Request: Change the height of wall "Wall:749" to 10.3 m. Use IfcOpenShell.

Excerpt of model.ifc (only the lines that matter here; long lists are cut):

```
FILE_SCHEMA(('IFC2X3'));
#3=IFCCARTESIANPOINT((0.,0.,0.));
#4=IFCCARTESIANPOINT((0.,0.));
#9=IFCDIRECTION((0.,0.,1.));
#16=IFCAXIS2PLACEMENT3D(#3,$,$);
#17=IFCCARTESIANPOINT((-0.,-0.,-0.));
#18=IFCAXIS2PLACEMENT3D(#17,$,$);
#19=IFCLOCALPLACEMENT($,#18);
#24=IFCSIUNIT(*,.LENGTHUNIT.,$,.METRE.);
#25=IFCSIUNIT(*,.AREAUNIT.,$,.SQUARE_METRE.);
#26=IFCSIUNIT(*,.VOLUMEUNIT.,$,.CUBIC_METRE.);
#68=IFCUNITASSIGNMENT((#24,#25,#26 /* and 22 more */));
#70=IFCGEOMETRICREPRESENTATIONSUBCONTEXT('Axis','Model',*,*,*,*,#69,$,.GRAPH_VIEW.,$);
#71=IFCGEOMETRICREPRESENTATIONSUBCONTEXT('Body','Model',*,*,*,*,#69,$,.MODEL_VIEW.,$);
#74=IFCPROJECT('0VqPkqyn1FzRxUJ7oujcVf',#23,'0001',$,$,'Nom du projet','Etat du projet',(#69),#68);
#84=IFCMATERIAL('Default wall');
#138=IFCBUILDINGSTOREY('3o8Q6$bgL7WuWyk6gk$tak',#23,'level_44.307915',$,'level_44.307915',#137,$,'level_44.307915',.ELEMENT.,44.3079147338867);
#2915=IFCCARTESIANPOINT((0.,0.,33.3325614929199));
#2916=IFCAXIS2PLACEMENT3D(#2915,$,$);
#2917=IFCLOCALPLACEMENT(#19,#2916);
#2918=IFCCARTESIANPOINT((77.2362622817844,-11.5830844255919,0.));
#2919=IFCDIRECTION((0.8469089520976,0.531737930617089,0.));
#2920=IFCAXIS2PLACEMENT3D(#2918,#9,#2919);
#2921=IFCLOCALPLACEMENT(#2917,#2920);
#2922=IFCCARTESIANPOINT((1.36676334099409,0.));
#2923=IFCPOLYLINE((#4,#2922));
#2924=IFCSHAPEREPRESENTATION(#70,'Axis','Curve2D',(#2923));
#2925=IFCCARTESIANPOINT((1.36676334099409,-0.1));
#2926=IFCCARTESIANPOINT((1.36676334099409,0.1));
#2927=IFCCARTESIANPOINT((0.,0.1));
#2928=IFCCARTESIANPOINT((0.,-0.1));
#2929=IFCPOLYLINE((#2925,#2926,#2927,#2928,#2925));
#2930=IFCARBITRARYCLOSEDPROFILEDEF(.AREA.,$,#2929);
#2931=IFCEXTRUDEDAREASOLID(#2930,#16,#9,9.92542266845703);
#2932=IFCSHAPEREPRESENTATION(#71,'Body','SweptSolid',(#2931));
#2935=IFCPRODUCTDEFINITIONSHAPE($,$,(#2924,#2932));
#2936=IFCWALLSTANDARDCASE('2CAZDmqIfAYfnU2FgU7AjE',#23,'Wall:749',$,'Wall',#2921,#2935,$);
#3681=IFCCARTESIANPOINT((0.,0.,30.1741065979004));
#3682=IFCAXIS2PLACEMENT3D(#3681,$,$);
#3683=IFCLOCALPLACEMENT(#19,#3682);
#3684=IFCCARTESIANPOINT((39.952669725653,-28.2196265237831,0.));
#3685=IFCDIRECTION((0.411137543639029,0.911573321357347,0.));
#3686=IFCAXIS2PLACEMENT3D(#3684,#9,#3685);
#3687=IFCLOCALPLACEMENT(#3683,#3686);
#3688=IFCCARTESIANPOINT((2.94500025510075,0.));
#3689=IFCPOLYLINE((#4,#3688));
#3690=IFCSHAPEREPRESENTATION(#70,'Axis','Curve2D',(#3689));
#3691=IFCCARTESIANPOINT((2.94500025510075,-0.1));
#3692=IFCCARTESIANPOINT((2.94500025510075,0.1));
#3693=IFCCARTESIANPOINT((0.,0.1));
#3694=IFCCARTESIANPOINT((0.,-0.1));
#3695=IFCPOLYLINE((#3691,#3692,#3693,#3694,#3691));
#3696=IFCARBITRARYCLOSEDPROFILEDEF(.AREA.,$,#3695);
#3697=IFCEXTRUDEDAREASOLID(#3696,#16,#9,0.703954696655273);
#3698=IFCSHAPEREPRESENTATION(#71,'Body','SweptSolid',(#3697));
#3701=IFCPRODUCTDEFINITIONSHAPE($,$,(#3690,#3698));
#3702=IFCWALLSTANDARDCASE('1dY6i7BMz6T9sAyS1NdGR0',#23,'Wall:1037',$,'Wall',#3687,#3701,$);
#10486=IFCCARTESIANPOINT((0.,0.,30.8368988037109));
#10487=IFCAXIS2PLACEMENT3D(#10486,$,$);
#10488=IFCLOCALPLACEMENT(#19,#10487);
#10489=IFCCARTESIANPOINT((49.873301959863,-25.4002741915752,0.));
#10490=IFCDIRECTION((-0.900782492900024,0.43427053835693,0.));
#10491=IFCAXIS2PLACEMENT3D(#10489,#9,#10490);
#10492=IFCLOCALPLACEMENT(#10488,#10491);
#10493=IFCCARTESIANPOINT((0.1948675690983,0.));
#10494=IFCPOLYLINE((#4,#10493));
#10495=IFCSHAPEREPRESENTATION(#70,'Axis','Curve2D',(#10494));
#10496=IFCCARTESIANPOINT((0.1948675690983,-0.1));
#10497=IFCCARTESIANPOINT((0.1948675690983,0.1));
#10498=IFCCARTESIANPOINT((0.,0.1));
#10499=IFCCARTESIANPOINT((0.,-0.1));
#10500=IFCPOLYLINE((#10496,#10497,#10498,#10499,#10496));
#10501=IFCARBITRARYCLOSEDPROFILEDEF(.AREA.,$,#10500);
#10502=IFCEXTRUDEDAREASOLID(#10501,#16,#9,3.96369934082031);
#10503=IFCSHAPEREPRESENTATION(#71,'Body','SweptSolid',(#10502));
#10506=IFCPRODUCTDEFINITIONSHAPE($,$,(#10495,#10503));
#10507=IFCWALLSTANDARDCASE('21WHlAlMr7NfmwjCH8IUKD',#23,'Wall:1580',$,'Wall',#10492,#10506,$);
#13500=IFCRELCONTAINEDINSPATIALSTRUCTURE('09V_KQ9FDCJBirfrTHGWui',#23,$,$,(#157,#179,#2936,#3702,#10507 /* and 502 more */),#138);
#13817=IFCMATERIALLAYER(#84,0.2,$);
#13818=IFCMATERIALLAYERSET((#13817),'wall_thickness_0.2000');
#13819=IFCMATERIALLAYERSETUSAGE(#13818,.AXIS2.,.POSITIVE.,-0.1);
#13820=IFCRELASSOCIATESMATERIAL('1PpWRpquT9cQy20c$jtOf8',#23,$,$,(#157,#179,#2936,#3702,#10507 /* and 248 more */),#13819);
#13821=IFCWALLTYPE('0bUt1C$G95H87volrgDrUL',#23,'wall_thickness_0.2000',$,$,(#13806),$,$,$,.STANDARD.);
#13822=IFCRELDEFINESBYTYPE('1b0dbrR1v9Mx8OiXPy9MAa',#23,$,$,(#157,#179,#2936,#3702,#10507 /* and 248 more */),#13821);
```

```python
import ifcopenshell
import ifcopenshell.geom
import ifcopenshell.util.representation
import ifcopenshell.util.shape
import ifcopenshell.util.unit

model = ifcopenshell.open("model.ifc")
unit_scale = ifcopenshell.util.unit.calculate_unit_scale(model)
settings = ifcopenshell.geom.settings()


def volume(element):
    """Net volume in cubic metres, openings subtracted."""
    shape = ifcopenshell.geom.create_shape(settings, element)
    return ifcopenshell.util.shape.get_volume(shape.geometry)


wall = model.by_guid("2CAZDmqIfAYfnU2FgU7AjE")
before = volume(wall)

body = ifcopenshell.util.representation.get_representation(wall, "Model", "Body")
solid = body.Items[0]
old_height = solid.Depth
solid.Depth = 10.3 / unit_scale
after = volume(wall)

print(f"height {old_height:g} -> {solid.Depth:g}, volume {before:.3f} -> {after:.3f} m3")

model.write("model_updated.ifc")
```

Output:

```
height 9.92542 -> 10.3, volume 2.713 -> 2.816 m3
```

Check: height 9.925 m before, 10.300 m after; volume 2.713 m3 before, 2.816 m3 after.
